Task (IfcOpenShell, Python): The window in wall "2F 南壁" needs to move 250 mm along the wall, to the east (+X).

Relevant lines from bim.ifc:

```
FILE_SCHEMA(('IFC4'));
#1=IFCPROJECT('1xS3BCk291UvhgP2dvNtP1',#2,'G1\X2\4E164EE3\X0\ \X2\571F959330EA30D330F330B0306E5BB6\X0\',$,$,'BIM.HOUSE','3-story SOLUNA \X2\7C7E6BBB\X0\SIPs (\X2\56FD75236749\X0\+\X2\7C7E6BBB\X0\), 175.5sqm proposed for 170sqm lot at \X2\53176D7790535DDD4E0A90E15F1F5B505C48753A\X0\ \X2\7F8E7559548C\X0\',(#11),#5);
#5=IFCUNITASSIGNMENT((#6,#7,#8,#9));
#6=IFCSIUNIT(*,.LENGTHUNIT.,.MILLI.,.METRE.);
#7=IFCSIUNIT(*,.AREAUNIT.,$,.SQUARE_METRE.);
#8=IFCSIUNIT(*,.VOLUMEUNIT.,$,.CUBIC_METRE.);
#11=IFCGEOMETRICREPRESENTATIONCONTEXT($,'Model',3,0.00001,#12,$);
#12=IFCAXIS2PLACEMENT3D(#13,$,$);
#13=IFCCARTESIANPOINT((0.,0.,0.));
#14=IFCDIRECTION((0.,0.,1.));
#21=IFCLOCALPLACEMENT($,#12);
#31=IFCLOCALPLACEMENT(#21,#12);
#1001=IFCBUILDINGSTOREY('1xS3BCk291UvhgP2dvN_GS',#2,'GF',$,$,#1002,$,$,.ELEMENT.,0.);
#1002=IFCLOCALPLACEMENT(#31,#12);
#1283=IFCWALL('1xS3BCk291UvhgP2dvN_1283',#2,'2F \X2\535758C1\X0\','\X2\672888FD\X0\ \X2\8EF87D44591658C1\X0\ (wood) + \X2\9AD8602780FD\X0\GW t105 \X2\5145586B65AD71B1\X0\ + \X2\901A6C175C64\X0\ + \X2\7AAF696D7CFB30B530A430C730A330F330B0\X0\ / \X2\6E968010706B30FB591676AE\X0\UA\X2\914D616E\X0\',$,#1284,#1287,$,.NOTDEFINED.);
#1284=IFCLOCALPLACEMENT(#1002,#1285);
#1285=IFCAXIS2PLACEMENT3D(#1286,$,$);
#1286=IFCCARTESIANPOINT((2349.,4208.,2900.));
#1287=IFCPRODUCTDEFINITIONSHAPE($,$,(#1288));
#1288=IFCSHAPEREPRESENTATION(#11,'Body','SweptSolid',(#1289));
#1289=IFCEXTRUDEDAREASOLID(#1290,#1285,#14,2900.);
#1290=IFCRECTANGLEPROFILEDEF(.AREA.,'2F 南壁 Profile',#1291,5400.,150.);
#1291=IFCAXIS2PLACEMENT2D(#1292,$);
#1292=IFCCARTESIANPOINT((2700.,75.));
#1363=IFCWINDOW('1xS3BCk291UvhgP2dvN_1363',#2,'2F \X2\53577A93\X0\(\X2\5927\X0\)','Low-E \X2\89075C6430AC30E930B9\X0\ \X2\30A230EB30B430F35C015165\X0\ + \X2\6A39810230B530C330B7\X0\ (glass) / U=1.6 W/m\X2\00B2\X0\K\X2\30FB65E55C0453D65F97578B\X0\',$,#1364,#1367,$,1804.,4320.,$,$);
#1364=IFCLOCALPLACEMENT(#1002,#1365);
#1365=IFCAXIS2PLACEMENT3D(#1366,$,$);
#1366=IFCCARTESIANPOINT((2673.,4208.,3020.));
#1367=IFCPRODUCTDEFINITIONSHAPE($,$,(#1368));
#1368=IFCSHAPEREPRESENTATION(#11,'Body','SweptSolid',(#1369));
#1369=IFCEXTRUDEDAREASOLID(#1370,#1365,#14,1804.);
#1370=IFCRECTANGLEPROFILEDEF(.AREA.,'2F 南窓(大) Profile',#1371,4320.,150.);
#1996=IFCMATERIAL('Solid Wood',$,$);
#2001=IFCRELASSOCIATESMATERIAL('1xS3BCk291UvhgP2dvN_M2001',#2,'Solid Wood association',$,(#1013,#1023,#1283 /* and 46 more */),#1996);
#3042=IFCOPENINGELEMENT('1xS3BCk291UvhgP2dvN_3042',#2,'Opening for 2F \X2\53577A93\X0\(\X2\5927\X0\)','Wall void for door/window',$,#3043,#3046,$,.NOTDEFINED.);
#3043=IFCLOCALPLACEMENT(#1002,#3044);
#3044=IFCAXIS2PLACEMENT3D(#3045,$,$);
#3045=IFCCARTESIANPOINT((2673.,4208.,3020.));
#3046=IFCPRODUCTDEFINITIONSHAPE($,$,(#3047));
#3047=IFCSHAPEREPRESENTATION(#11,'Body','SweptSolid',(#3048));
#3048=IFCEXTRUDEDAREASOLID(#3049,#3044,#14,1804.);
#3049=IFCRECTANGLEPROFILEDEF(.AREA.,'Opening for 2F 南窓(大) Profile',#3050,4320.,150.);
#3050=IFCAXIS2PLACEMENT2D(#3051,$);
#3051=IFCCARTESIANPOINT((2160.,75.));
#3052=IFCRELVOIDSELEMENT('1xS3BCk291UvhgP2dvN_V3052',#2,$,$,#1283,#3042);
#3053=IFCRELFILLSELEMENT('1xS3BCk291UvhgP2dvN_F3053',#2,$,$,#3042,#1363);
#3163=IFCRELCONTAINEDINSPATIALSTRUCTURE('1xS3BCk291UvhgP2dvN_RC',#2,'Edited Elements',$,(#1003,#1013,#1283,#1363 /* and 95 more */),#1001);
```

```python
import ifcopenshell
import ifcopenshell.api.geometry
import ifcopenshell.util.placement

model = ifcopenshell.open("bim.ifc")

window = model.by_guid("1xS3BCk291UvhgP2dvN_1363")
opening = window.FillsVoids[0].RelatingOpeningElement
wall = opening.VoidsElements[0].RelatingBuildingElement

wall_matrix = ifcopenshell.util.placement.get_local_placement(wall.ObjectPlacement)
shift = wall_matrix[:3, 0] * 250.0
before = ifcopenshell.util.placement.get_local_placement(window.ObjectPlacement)[:3, 3].copy()

# The window is not placed relative to its opening, so move both.
for product in (opening, window):
    matrix = ifcopenshell.util.placement.get_local_placement(product.ObjectPlacement)
    matrix[:3, 3] += shift
    ifcopenshell.api.geometry.edit_object_placement(model, product=product, matrix=matrix, is_si=False)

after = ifcopenshell.util.placement.get_local_placement(window.ObjectPlacement)[:3, 3]
print("window moved by", (after - before).round(3) + 0.0)

model.write("bim_updated.ifc")
```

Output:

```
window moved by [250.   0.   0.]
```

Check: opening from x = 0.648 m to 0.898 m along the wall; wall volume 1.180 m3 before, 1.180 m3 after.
